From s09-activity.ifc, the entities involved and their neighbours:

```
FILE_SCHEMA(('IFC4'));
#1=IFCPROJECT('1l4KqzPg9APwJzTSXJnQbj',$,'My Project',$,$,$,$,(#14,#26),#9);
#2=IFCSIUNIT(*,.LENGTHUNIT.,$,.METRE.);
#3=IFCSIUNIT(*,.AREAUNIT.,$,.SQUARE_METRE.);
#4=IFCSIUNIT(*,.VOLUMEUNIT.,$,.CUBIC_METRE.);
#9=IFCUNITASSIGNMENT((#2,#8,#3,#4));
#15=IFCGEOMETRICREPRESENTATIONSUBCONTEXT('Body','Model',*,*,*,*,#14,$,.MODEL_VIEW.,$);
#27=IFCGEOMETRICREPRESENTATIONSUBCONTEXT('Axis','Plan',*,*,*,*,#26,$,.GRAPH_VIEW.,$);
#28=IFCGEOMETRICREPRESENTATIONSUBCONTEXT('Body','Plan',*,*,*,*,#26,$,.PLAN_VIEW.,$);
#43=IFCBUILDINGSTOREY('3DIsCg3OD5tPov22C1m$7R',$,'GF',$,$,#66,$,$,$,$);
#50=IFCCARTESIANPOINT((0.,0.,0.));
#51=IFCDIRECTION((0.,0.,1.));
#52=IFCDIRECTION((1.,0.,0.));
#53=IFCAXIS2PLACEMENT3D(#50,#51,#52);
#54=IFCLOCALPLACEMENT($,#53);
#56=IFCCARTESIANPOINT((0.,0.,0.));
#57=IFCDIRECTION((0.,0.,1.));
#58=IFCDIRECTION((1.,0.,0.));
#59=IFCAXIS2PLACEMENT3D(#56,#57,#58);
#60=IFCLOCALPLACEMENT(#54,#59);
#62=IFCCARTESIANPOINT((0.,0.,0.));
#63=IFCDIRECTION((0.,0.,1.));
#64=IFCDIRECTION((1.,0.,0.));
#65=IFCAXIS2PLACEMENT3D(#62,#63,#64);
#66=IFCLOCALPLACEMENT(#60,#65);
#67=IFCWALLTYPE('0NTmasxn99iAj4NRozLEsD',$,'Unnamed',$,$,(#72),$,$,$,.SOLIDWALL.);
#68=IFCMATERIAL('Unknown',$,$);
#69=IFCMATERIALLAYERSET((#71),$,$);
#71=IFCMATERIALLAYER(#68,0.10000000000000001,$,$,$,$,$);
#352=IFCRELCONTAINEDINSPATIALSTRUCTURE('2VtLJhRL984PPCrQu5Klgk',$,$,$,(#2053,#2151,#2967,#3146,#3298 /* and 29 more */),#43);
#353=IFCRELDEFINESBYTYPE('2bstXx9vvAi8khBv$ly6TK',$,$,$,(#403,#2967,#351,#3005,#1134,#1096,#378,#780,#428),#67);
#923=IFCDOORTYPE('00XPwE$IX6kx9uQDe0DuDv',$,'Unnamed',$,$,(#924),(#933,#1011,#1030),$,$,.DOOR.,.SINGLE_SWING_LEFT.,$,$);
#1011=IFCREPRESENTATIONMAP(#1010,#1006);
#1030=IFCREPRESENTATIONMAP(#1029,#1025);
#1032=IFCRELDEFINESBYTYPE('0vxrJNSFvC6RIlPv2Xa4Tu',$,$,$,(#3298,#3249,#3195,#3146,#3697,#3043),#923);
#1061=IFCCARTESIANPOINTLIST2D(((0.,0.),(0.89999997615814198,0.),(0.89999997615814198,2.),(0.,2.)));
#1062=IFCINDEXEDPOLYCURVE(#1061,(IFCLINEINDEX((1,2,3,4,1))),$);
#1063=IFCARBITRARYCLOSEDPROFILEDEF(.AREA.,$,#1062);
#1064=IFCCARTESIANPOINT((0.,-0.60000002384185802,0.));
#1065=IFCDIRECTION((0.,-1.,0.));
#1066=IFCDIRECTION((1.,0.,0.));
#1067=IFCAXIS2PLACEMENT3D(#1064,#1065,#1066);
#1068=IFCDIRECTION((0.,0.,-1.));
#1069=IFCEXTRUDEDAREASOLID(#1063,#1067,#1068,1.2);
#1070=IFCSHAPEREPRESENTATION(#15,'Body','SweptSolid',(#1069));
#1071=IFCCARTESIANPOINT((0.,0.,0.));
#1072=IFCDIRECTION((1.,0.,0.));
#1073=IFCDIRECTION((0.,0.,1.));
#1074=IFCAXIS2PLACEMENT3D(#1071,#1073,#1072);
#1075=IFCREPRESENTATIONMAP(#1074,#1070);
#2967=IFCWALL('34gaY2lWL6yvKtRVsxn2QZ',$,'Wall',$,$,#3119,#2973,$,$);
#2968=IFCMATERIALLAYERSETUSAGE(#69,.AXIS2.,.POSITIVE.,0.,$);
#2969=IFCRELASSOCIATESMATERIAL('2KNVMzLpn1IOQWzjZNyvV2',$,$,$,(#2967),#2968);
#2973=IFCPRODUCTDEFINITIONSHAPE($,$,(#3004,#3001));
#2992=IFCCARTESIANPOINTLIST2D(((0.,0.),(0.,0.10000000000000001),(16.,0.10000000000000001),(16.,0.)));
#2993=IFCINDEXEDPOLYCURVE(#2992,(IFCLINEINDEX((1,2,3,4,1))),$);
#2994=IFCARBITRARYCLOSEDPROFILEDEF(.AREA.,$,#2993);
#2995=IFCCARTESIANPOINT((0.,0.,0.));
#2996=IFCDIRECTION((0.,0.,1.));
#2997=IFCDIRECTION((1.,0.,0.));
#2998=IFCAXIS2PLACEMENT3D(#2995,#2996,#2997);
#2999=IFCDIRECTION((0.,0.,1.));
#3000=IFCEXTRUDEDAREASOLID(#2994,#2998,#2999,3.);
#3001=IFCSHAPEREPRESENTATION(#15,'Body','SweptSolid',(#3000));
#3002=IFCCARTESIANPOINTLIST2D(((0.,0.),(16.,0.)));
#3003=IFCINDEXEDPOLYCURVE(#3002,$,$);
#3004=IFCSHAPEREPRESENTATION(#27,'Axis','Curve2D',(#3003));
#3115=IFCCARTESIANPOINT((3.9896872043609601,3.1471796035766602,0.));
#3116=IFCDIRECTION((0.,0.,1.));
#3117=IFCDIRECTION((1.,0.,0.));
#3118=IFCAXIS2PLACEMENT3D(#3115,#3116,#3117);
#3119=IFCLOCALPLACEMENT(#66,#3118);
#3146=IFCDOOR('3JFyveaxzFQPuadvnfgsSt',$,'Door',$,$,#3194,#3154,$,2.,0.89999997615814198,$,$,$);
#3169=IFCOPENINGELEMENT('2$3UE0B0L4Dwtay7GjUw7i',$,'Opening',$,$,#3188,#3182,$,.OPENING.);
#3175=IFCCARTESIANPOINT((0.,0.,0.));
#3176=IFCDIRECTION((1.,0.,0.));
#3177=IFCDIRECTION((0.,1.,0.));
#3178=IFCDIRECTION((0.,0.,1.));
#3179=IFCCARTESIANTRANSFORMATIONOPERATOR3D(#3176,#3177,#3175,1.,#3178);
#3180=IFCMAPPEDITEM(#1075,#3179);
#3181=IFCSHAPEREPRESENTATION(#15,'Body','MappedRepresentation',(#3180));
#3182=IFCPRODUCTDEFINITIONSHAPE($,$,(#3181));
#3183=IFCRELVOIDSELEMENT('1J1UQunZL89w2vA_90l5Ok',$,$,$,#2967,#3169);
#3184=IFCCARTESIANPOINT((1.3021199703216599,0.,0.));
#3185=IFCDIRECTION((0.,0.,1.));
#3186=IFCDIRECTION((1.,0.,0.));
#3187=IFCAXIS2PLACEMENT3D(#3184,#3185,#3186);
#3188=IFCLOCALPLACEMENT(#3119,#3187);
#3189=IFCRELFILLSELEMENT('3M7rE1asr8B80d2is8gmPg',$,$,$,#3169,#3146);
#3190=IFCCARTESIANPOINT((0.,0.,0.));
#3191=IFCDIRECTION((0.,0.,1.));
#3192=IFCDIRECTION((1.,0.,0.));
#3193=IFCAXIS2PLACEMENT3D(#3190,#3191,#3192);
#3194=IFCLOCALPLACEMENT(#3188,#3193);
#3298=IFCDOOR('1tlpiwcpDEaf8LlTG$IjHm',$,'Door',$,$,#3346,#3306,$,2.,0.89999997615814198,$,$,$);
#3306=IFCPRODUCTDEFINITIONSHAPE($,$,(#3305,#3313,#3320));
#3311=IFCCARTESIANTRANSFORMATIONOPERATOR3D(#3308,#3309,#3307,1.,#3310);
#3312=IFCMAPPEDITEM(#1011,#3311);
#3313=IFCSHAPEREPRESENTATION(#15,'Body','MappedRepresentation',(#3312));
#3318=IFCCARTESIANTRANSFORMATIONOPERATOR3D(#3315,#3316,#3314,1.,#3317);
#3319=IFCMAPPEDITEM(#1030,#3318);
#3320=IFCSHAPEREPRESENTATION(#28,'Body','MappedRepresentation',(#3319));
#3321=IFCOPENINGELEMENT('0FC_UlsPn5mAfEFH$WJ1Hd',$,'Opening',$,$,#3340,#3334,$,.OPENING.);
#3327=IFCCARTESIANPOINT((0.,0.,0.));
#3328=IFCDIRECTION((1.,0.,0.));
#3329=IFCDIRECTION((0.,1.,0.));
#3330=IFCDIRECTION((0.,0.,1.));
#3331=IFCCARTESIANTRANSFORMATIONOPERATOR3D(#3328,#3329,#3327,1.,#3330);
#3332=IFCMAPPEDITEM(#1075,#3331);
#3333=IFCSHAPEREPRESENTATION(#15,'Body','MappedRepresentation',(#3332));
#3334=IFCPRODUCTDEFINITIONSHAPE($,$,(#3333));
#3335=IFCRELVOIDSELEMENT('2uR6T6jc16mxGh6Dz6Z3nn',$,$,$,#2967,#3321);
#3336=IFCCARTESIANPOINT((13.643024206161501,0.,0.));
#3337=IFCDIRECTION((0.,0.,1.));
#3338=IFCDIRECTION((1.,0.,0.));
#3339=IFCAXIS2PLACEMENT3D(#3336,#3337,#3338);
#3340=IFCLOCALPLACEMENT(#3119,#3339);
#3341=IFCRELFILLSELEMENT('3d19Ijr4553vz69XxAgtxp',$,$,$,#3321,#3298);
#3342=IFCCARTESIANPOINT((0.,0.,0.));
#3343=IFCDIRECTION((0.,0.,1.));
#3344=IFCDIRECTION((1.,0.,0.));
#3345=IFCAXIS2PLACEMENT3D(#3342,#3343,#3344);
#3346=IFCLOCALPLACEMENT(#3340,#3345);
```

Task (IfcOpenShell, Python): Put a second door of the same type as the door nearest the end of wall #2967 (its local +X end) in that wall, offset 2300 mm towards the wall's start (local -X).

```python
import ifcopenshell
import ifcopenshell.api.feature
import ifcopenshell.api.geometry
import ifcopenshell.api.root
import ifcopenshell.geom
import ifcopenshell.util.element
import ifcopenshell.util.placement
import ifcopenshell.util.shape

model = ifcopenshell.open("s09-activity.ifc")
settings = ifcopenshell.geom.settings()


def volume(element):
    """Net volume in cubic metres, openings subtracted."""
    shape = ifcopenshell.geom.create_shape(settings, element)
    return ifcopenshell.util.shape.get_volume(shape.geometry)


door = model.by_id(3298)
opening = door.FillsVoids[0].RelatingOpeningElement
wall = opening.VoidsElements[0].RelatingBuildingElement
before = volume(wall)
shift = ifcopenshell.util.placement.get_local_placement(wall.ObjectPlacement)[:3, 0] * -2.3

# copy_class copies the void relationship, type, container and properties, but no geometry.
new_opening = ifcopenshell.api.root.copy_class(model, product=opening)
new_opening.Representation = ifcopenshell.util.element.copy_deep(
    model, opening.Representation, exclude=["IfcGeometricRepresentationContext", "IfcRepresentationMap"]
)
new_door = ifcopenshell.api.root.copy_class(model, product=door)
new_door.Representation = ifcopenshell.util.element.copy_deep(
    model, door.Representation, exclude=["IfcGeometricRepresentationContext", "IfcRepresentationMap"]
)
ifcopenshell.api.feature.add_filling(model, opening=new_opening, element=new_door)

for old, new in ((opening, new_opening), (door, new_door)):
    matrix = ifcopenshell.util.placement.get_local_placement(old.ObjectPlacement)
    matrix[:3, 3] += shift
    ifcopenshell.api.geometry.edit_object_placement(model, product=new, matrix=matrix, is_si=False)

after = volume(wall)

print(f"wall volume {before:.3f} -> {after:.3f} m3")

model.write("s09-activity_v2.ifc")
```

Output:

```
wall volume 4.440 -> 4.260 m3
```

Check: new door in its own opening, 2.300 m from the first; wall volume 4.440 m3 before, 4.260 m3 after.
